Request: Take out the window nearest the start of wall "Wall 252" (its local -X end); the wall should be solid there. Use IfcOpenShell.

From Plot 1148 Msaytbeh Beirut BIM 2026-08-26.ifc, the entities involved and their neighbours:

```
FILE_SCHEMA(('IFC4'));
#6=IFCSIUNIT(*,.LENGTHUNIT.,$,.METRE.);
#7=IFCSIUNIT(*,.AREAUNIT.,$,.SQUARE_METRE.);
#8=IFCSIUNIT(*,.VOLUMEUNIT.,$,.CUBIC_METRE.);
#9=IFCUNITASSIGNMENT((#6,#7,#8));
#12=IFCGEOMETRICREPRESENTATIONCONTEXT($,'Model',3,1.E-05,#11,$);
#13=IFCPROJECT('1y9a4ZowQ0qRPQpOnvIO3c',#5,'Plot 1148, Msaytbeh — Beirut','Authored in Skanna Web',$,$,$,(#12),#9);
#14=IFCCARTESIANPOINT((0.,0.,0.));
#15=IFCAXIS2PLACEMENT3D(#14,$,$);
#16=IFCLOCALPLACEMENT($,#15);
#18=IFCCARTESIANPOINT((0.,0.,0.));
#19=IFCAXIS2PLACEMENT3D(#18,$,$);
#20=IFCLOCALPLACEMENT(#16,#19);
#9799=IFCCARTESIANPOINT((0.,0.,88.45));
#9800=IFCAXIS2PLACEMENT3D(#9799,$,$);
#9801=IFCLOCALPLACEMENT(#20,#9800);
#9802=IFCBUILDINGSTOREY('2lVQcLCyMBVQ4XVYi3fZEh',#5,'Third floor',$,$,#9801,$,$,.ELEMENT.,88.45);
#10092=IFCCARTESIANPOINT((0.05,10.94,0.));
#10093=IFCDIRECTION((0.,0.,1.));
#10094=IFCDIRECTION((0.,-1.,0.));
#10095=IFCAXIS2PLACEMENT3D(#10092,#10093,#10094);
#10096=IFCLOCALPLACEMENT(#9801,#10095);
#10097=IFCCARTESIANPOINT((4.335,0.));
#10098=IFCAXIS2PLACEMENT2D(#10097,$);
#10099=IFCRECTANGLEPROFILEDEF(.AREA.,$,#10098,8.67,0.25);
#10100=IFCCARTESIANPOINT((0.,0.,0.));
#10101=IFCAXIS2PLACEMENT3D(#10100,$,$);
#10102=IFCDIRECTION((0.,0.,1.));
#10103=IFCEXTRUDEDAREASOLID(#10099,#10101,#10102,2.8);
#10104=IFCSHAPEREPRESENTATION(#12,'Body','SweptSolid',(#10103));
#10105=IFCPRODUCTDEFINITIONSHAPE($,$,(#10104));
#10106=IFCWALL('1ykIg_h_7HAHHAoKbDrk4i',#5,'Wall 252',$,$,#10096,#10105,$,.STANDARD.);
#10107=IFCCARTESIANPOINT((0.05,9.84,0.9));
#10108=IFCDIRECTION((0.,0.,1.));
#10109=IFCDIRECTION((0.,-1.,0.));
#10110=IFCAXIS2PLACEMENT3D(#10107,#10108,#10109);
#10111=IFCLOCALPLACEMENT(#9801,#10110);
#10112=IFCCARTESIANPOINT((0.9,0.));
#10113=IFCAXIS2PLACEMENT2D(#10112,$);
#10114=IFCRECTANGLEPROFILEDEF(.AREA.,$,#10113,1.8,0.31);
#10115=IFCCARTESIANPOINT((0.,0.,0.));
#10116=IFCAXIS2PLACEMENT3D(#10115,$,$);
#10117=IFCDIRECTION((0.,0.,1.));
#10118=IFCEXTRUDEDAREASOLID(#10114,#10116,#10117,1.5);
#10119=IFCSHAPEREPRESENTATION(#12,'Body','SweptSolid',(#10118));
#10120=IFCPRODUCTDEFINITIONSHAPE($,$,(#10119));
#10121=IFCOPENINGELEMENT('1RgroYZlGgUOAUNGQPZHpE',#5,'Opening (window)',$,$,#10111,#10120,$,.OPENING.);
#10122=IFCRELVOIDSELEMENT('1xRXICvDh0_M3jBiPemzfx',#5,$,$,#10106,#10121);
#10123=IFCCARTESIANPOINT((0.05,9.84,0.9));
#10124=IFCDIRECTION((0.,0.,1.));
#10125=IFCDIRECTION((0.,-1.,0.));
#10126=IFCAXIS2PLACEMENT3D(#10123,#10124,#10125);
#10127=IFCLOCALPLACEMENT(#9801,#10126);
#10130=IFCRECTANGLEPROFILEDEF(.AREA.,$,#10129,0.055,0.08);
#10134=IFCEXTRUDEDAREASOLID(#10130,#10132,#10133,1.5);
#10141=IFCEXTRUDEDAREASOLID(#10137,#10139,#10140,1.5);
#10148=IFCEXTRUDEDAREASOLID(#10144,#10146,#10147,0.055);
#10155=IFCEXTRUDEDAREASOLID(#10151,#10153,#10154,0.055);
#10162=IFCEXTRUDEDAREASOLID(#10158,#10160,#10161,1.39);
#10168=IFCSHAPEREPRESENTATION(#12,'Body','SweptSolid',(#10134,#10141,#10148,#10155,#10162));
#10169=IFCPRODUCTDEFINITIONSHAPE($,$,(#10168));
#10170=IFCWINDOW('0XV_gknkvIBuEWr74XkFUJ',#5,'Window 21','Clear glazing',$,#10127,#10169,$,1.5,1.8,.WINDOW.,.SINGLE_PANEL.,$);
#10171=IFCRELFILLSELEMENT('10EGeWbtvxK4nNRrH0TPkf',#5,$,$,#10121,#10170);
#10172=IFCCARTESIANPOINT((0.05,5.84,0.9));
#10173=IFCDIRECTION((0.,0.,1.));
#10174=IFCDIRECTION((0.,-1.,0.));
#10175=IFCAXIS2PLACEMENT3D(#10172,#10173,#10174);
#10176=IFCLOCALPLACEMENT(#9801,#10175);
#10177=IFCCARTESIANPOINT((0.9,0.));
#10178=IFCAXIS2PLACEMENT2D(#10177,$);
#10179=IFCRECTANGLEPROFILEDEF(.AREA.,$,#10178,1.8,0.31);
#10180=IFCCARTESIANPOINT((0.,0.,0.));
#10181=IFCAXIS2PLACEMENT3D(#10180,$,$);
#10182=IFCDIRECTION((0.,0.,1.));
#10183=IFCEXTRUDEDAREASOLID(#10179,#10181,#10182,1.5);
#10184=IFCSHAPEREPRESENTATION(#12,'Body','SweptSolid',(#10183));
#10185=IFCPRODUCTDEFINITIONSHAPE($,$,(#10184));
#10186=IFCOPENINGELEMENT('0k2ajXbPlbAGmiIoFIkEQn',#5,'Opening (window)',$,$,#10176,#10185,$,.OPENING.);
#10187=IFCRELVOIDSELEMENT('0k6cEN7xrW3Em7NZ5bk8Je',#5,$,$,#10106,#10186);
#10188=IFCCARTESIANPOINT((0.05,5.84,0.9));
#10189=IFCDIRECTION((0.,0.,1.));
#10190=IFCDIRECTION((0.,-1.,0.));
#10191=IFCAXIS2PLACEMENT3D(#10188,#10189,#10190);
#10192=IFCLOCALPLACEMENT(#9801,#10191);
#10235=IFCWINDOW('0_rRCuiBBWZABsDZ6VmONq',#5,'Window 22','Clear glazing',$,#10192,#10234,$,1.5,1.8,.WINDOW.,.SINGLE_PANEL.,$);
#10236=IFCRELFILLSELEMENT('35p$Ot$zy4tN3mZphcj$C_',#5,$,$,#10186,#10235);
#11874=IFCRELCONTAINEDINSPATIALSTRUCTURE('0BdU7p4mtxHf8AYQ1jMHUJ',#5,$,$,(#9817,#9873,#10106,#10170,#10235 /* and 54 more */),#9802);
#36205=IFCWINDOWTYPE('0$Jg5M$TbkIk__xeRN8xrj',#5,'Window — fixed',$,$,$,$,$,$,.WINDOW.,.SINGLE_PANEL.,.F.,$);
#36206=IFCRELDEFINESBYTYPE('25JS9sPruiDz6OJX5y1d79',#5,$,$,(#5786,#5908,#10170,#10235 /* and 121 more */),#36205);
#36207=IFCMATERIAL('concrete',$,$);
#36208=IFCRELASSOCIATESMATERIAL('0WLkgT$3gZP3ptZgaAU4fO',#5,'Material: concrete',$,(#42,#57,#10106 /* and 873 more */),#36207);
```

```python
import ifcopenshell
import ifcopenshell.api.feature
import ifcopenshell.api.root
import ifcopenshell.geom
import ifcopenshell.util.shape

model = ifcopenshell.open("Plot 1148 Msaytbeh Beirut BIM 2026-08-26.ifc")
settings = ifcopenshell.geom.settings()


def volume(element):
    """Net volume in cubic metres, openings subtracted."""
    shape = ifcopenshell.geom.create_shape(settings, element)
    return ifcopenshell.util.shape.get_volume(shape.geometry)


window = model.by_guid("0XV_gknkvIBuEWr74XkFUJ")
opening = window.FillsVoids[0].RelatingOpeningElement
wall = opening.VoidsElements[0].RelatingBuildingElement
before = volume(wall)

ifcopenshell.api.root.remove_product(model, product=window)
ifcopenshell.api.feature.remove_feature(model, feature=opening)

after = volume(wall)

print(f"wall volume {before:.3f} -> {after:.3f} m3")

model.write("Plot 1148 Msaytbeh Beirut BIM 2026-08-26-out.ifc")
```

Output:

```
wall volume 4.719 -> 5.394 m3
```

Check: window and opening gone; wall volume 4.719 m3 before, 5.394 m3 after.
